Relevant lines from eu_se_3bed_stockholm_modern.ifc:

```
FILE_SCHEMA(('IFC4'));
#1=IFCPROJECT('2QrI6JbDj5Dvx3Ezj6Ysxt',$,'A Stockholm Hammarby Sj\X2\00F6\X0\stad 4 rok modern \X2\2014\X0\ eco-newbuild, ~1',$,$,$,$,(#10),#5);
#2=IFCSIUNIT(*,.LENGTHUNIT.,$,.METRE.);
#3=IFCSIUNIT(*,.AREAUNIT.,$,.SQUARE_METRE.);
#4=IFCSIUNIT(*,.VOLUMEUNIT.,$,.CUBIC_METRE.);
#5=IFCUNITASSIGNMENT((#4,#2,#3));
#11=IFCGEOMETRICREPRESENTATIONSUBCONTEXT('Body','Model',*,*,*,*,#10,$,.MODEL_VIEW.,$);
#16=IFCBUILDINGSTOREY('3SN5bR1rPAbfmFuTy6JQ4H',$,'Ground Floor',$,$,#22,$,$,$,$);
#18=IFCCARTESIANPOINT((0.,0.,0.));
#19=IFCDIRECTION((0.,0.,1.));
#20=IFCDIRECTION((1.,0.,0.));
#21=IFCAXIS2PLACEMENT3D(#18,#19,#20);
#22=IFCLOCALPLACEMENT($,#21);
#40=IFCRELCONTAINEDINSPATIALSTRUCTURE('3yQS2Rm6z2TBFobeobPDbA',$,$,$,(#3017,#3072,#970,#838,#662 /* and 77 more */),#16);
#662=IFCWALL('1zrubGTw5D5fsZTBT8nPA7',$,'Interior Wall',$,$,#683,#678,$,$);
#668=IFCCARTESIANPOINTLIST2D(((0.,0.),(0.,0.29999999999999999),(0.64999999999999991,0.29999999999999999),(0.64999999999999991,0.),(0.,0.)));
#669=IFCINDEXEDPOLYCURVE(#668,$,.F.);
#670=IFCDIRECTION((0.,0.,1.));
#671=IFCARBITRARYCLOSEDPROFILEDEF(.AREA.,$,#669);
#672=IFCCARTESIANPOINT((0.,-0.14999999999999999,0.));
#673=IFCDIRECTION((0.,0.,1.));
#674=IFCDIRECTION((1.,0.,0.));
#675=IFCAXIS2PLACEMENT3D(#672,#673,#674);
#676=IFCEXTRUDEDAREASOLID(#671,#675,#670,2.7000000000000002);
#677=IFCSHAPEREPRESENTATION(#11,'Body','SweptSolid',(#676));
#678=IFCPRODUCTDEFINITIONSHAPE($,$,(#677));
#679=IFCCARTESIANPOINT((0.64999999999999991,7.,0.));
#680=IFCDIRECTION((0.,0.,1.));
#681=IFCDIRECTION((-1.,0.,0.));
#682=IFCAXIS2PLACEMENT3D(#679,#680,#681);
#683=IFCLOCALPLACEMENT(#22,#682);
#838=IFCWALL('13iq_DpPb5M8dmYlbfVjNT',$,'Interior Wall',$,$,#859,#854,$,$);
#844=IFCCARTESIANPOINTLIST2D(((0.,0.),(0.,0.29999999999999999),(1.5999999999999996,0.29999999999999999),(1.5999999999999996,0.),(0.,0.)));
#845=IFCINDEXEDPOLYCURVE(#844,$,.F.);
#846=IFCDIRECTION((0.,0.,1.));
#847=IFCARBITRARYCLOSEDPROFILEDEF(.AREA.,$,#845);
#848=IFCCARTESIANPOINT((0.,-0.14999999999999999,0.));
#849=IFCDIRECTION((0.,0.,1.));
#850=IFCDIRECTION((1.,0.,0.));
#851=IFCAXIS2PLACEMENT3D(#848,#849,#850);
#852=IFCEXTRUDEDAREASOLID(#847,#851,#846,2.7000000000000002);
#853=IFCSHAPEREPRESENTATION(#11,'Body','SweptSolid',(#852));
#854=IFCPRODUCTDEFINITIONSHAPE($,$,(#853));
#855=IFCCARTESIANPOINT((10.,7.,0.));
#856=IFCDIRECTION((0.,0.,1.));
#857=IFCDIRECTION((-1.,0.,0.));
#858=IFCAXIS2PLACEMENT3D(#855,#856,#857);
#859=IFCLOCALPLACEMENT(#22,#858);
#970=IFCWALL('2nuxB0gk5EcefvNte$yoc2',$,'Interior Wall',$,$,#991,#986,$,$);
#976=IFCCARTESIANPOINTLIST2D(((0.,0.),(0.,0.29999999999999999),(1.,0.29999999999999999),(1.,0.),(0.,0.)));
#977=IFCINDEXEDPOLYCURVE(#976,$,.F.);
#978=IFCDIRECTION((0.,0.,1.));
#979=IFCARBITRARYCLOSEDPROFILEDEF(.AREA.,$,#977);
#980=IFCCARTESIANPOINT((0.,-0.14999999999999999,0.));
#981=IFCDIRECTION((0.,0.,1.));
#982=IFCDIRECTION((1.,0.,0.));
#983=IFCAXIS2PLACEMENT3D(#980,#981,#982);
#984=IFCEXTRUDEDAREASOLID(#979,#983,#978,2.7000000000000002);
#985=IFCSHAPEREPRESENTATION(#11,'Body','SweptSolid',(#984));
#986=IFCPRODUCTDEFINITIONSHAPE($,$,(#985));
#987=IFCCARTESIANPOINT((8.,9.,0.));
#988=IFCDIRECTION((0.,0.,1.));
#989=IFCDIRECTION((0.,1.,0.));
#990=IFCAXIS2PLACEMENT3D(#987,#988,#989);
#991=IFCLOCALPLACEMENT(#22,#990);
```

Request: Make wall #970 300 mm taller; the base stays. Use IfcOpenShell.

```python
import ifcopenshell
import ifcopenshell.geom
import ifcopenshell.util.representation
import ifcopenshell.util.shape
import ifcopenshell.util.unit

model = ifcopenshell.open("eu_se_3bed_stockholm_modern.ifc")
unit_scale = ifcopenshell.util.unit.calculate_unit_scale(model)
settings = ifcopenshell.geom.settings()


def volume(element):
    """Net volume in cubic metres, openings subtracted."""
    shape = ifcopenshell.geom.create_shape(settings, element)
    return ifcopenshell.util.shape.get_volume(shape.geometry)


wall = model.by_guid("2nuxB0gk5EcefvNte$yoc2")
before = volume(wall)

body = ifcopenshell.util.representation.get_representation(wall, "Model", "Body")
solid = body.Items[0]
old_height = solid.Depth
solid.Depth += 0.3 / unit_scale
after = volume(wall)

print(f"height {old_height:g} -> {solid.Depth:g}, volume {before:.3f} -> {after:.3f} m3")

model.write("eu_se_3bed_stockholm_modern_v2.ifc")
```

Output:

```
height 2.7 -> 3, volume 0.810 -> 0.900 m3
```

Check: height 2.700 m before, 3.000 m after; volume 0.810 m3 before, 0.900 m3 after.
